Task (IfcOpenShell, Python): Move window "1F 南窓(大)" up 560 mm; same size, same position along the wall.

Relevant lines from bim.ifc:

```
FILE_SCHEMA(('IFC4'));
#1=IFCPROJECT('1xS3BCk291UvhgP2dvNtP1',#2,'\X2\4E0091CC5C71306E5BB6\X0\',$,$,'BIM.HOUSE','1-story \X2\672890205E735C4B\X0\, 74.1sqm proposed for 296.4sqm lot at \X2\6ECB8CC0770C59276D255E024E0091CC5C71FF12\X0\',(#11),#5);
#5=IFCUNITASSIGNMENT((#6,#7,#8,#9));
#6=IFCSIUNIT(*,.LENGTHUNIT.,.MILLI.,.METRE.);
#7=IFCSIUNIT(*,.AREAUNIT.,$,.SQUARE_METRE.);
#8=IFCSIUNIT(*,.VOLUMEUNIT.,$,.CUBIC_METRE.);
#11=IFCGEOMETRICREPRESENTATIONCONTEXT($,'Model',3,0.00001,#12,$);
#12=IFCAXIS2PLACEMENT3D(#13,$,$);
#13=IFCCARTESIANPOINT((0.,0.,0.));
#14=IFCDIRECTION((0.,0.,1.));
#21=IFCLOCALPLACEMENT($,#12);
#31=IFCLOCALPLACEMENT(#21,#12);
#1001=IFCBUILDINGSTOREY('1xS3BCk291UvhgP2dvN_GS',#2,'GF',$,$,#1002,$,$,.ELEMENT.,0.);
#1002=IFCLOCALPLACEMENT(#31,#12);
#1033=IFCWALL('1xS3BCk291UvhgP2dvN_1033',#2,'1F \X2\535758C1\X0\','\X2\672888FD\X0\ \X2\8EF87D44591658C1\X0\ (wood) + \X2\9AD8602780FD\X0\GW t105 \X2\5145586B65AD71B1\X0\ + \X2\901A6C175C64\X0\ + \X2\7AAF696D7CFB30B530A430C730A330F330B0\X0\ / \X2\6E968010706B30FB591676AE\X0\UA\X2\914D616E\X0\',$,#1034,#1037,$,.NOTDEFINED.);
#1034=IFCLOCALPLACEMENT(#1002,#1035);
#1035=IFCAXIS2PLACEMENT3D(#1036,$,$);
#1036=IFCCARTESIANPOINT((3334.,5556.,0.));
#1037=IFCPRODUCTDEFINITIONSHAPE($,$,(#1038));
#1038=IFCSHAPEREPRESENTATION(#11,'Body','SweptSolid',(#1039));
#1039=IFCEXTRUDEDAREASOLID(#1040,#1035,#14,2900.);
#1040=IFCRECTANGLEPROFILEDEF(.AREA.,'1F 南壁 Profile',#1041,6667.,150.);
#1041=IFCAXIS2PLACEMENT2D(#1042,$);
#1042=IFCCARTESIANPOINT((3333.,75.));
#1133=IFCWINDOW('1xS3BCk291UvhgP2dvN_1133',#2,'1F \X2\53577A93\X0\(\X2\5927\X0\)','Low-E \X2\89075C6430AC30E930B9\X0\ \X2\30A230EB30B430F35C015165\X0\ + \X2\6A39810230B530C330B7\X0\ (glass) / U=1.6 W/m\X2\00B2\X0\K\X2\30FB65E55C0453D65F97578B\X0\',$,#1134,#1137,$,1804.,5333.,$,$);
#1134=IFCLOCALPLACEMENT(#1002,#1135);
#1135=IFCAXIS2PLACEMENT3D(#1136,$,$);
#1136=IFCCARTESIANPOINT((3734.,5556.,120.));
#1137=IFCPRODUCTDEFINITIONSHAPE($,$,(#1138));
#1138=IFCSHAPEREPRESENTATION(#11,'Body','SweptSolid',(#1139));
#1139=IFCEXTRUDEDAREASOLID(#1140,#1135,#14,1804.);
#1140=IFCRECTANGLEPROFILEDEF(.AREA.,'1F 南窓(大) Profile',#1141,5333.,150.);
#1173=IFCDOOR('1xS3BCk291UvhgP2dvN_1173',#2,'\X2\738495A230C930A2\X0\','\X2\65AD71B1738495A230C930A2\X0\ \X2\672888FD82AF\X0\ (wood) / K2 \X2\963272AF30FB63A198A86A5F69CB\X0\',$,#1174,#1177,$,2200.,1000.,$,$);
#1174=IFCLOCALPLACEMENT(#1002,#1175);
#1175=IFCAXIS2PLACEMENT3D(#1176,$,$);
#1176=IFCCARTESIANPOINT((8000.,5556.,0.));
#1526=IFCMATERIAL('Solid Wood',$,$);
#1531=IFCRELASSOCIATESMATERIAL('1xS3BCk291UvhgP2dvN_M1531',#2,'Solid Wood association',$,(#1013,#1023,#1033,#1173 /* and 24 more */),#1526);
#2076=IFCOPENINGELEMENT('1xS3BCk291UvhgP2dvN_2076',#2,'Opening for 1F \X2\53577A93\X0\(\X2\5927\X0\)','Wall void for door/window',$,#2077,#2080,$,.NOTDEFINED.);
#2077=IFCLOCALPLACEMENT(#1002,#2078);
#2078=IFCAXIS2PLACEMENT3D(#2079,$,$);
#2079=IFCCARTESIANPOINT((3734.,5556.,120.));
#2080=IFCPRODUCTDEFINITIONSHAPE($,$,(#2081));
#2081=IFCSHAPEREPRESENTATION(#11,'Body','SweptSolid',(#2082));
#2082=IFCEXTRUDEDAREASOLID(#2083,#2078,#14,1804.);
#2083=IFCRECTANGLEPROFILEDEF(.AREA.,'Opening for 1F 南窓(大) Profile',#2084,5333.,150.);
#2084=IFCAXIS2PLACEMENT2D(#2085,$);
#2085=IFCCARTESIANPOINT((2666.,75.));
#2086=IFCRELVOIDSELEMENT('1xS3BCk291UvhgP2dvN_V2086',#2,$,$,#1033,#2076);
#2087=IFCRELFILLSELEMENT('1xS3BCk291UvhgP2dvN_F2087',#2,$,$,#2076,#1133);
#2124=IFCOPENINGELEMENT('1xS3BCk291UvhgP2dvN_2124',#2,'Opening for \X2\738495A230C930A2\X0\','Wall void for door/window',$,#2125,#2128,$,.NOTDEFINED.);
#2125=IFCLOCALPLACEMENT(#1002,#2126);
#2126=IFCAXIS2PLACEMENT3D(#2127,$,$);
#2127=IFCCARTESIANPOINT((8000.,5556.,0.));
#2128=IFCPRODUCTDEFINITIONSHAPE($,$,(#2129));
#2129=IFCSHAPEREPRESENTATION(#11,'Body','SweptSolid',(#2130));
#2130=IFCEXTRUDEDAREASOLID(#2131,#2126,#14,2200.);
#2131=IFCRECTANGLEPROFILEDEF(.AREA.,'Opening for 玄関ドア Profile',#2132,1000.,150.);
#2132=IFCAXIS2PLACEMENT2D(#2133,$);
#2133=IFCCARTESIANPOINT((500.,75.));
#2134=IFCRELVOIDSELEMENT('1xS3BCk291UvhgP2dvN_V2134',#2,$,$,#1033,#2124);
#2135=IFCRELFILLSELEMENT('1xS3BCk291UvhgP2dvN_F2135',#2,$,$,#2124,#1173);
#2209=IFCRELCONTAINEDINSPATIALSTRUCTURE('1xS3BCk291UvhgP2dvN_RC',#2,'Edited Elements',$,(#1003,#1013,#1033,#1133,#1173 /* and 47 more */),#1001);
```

```python
import numpy as np
import ifcopenshell
import ifcopenshell.api.geometry
import ifcopenshell.util.placement
import ifcopenshell.util.unit

model = ifcopenshell.open("bim.ifc")
unit_scale = ifcopenshell.util.unit.calculate_unit_scale(model)

window = model.by_id(1133)
opening = window.FillsVoids[0].RelatingOpeningElement
dz = 0.56 / unit_scale

shift = np.array([0.0, 0.0, dz])
# The window is not placed relative to its opening, so move both.
for product in (opening, window):
    matrix = ifcopenshell.util.placement.get_local_placement(product.ObjectPlacement)
    matrix[:3, 3] += shift
    ifcopenshell.api.geometry.edit_object_placement(model, product=product, matrix=matrix, is_si=False)

print(f"moved by {dz * unit_scale:+.3f} m")

model.write("bim_rev.ifc")
```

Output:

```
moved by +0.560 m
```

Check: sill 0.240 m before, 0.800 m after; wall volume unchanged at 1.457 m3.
